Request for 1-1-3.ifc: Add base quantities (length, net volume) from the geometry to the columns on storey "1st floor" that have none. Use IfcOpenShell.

First a look at what the model holds.

```python
import ifcopenshell
import ifcopenshell.util.element
import ifcopenshell.util.unit

model = ifcopenshell.open("1-1-3.ifc")
print(model.schema)
for unit_type in ("LENGTHUNIT", "AREAUNIT", "VOLUMEUNIT"):
    print(unit_type, ifcopenshell.util.unit.calculate_unit_scale(model, unit_type))
storey = next(s for s in model.by_type("IfcBuildingStorey") if s.Name == "1st floor")
columns = [e for e in ifcopenshell.util.element.get_decomposition(storey) if e.is_a("IfcColumn")]
for e in sorted(columns, key=lambda e: e.id()):
    print(e.id(), e.is_a(), e.Name, list(ifcopenshell.util.element.get_psets(e, qtos_only=True)), sep=" | ")
```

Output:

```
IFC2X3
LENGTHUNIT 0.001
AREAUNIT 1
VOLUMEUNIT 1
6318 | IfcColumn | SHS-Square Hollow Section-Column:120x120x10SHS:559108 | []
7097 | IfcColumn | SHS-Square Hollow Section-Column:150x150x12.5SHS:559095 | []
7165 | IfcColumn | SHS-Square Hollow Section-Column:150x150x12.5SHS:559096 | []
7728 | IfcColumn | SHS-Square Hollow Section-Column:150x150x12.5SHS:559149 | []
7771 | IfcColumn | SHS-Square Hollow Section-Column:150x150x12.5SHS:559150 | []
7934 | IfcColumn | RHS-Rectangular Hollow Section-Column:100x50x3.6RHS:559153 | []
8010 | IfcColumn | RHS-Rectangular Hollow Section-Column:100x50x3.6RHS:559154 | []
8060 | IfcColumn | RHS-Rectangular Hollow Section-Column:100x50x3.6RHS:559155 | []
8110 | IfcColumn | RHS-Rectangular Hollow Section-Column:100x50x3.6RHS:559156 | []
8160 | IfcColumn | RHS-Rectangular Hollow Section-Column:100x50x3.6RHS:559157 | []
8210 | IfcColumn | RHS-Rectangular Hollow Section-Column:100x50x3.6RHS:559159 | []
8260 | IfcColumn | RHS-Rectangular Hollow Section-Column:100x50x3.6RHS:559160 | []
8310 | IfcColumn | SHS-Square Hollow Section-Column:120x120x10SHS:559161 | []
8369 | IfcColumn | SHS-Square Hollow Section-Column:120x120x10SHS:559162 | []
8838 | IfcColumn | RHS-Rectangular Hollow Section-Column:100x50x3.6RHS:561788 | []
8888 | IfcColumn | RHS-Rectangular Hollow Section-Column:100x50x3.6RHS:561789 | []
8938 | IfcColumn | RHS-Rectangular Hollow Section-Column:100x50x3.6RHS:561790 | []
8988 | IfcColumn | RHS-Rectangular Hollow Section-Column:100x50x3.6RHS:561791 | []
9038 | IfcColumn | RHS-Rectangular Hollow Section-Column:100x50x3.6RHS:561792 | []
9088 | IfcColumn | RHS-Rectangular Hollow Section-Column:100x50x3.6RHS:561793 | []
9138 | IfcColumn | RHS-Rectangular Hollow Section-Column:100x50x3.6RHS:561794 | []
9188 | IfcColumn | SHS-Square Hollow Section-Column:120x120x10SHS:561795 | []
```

```python
import ifcopenshell
import ifcopenshell.api.pset
import ifcopenshell.geom
import ifcopenshell.util.element
import ifcopenshell.util.shape
import ifcopenshell.util.unit

model = ifcopenshell.open("1-1-3.ifc")
unit_scale = ifcopenshell.util.unit.calculate_unit_scale(model)
volume_scale = ifcopenshell.util.unit.calculate_unit_scale(model, "VOLUMEUNIT")
settings = ifcopenshell.geom.settings()

storey = next(s for s in model.by_type("IfcBuildingStorey") if s.Name == "1st floor")
columns = [e for e in ifcopenshell.util.element.get_decomposition(storey) if e.is_a("IfcColumn")]

for e in sorted(columns, key=lambda e: e.id()):
    if ifcopenshell.util.element.get_psets(e, qtos_only=True, should_inherit=False):
        continue
    # Geometry comes back in metres, in the element's own axes.
    shape = ifcopenshell.geom.create_shape(settings, e)
    values = {
        "Length": ifcopenshell.util.shape.get_z(shape.geometry) / unit_scale,
        "NetVolume": ifcopenshell.util.shape.get_volume(shape.geometry) / volume_scale,
    }
    qto = ifcopenshell.api.pset.add_qto(model, product=e, name="BaseQuantities")
    ifcopenshell.api.pset.edit_qto(model, qto=qto, properties=values)
    print(e.id(), {k: round(v, 3) for k, v in values.items()})

model.write("1-1-3_rev.ifc")
```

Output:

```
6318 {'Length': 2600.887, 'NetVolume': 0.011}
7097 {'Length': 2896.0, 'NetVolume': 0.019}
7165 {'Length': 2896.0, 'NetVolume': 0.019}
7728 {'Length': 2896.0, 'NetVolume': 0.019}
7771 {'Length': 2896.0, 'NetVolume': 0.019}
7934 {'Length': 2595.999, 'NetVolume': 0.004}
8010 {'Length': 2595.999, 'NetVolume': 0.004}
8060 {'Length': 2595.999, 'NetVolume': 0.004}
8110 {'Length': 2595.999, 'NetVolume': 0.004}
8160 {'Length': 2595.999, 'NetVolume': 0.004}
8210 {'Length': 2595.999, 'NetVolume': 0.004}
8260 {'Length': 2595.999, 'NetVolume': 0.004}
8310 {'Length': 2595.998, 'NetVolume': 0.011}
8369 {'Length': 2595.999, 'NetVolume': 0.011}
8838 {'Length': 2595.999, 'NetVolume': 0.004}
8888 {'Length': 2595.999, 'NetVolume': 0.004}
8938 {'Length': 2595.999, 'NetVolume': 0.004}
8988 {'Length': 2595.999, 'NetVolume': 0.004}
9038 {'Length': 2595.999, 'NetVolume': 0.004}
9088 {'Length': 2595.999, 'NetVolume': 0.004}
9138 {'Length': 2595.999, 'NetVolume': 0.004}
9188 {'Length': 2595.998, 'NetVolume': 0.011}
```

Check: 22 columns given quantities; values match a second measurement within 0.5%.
